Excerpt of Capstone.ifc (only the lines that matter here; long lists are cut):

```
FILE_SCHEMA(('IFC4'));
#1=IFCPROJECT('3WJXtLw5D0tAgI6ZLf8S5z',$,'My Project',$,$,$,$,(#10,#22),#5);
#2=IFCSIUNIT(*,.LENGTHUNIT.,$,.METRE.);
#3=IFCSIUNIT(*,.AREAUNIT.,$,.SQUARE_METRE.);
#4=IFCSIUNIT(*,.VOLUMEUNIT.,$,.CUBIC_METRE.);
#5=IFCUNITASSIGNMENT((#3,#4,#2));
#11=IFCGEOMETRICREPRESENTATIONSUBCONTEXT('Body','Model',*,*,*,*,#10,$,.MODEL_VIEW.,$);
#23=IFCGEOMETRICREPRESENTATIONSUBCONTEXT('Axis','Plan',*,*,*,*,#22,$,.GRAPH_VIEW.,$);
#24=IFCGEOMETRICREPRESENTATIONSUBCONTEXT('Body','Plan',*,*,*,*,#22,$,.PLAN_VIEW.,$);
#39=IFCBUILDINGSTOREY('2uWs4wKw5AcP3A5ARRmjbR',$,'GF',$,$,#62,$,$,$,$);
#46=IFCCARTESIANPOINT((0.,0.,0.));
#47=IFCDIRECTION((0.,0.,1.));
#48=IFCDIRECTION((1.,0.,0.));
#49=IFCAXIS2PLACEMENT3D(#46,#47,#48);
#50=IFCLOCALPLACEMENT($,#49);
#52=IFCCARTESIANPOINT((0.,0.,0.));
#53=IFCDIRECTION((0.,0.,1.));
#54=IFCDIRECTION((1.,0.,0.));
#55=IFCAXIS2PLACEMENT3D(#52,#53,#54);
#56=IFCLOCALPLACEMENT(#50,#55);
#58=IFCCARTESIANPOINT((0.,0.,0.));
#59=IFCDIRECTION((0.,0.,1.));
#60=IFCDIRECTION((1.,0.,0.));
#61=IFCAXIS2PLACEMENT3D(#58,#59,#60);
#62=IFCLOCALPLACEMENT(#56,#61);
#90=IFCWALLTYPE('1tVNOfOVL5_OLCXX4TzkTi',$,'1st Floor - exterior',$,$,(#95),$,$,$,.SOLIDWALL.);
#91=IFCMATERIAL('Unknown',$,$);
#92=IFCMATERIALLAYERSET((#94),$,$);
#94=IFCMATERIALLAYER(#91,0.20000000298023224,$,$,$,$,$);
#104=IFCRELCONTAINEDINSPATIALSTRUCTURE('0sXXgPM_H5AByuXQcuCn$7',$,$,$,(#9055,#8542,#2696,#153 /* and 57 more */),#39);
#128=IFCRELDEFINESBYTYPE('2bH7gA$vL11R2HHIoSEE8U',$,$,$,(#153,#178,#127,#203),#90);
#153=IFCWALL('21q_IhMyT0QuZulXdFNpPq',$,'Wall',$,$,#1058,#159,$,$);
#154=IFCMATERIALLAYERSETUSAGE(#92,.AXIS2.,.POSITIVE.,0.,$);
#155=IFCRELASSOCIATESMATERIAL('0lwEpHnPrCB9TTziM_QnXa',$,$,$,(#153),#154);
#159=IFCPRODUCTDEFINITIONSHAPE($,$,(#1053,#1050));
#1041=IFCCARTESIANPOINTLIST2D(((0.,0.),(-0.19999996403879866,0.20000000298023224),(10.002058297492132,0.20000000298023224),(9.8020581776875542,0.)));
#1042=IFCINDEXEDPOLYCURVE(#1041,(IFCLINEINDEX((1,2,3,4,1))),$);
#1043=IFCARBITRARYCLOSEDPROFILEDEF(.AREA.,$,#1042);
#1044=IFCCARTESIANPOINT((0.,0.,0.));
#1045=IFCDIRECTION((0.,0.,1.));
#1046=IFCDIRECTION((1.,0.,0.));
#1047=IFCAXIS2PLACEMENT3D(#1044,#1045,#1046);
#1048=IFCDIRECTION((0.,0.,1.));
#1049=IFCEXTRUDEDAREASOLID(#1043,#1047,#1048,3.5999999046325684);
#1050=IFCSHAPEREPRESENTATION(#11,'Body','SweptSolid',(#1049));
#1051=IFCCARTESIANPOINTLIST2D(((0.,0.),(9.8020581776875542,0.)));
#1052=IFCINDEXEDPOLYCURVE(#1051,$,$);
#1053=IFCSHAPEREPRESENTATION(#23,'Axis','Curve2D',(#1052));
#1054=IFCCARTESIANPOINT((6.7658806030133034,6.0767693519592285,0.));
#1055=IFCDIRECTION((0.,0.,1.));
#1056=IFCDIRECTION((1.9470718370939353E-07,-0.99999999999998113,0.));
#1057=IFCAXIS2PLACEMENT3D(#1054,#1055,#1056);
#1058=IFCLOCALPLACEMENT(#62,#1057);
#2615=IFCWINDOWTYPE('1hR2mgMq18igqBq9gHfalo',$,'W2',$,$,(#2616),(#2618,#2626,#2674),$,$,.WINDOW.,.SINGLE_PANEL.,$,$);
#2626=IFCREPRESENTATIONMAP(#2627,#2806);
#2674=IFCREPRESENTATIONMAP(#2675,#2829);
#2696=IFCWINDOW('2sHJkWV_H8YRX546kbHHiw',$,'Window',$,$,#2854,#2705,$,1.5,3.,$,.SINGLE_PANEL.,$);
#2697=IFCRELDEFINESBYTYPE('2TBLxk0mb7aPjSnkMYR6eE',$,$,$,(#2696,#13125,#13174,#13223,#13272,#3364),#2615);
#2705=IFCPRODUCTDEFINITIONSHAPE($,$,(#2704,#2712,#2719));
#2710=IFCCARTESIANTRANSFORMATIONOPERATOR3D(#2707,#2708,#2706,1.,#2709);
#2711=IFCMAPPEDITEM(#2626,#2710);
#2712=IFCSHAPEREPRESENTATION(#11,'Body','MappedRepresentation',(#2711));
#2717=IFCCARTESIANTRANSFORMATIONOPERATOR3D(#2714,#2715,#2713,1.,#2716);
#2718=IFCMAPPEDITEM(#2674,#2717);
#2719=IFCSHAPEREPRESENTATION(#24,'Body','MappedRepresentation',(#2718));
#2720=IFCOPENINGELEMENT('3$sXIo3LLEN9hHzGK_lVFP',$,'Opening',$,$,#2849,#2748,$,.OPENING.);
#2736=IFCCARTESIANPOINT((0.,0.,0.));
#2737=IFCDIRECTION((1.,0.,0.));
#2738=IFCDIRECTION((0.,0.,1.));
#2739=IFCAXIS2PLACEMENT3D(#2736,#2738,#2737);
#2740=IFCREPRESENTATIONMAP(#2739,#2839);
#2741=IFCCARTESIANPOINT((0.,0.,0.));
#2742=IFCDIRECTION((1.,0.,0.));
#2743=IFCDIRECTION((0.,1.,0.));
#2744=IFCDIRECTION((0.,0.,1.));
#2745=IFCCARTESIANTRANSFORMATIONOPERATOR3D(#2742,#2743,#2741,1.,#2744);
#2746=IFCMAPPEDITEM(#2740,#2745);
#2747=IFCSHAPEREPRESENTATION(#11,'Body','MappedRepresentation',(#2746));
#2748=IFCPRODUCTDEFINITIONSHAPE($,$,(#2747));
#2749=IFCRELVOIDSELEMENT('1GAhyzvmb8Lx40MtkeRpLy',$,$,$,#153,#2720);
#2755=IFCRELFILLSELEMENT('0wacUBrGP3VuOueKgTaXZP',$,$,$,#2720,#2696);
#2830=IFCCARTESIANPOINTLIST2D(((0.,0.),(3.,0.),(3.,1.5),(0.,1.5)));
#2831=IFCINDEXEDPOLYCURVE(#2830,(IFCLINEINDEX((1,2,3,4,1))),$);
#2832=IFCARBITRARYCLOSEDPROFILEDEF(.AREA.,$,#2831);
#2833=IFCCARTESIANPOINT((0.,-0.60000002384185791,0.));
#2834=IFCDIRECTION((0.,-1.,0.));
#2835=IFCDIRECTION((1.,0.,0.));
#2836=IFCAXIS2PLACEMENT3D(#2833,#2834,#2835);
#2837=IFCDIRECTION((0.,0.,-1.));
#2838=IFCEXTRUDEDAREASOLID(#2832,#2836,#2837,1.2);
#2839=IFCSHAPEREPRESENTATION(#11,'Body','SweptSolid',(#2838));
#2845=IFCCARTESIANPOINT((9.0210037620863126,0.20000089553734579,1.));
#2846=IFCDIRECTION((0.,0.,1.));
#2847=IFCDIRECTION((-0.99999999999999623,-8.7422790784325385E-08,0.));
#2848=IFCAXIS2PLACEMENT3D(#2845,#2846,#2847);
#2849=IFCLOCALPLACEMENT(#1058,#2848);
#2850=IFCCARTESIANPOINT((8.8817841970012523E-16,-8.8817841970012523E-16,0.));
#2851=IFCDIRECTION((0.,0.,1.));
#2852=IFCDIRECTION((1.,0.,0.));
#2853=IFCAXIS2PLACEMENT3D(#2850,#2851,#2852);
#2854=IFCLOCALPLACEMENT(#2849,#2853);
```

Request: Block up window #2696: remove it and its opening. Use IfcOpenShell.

```python
import ifcopenshell
import ifcopenshell.api.feature
import ifcopenshell.api.root
import ifcopenshell.geom
import ifcopenshell.util.shape

model = ifcopenshell.open("Capstone.ifc")
settings = ifcopenshell.geom.settings()


def volume(element):
    """Net volume in cubic metres, openings subtracted."""
    shape = ifcopenshell.geom.create_shape(settings, element)
    return ifcopenshell.util.shape.get_volume(shape.geometry)


window = model.by_guid("2sHJkWV_H8YRX546kbHHiw")
opening = window.FillsVoids[0].RelatingOpeningElement
wall = opening.VoidsElements[0].RelatingBuildingElement
before = volume(wall)

ifcopenshell.api.root.remove_product(model, product=window)
ifcopenshell.api.feature.remove_feature(model, feature=opening)

after = volume(wall)

print(f"wall volume {before:.3f} -> {after:.3f} m3")

model.write("Capstone_edited.ifc")
```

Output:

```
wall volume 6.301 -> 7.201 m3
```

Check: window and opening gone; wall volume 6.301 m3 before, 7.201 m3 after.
